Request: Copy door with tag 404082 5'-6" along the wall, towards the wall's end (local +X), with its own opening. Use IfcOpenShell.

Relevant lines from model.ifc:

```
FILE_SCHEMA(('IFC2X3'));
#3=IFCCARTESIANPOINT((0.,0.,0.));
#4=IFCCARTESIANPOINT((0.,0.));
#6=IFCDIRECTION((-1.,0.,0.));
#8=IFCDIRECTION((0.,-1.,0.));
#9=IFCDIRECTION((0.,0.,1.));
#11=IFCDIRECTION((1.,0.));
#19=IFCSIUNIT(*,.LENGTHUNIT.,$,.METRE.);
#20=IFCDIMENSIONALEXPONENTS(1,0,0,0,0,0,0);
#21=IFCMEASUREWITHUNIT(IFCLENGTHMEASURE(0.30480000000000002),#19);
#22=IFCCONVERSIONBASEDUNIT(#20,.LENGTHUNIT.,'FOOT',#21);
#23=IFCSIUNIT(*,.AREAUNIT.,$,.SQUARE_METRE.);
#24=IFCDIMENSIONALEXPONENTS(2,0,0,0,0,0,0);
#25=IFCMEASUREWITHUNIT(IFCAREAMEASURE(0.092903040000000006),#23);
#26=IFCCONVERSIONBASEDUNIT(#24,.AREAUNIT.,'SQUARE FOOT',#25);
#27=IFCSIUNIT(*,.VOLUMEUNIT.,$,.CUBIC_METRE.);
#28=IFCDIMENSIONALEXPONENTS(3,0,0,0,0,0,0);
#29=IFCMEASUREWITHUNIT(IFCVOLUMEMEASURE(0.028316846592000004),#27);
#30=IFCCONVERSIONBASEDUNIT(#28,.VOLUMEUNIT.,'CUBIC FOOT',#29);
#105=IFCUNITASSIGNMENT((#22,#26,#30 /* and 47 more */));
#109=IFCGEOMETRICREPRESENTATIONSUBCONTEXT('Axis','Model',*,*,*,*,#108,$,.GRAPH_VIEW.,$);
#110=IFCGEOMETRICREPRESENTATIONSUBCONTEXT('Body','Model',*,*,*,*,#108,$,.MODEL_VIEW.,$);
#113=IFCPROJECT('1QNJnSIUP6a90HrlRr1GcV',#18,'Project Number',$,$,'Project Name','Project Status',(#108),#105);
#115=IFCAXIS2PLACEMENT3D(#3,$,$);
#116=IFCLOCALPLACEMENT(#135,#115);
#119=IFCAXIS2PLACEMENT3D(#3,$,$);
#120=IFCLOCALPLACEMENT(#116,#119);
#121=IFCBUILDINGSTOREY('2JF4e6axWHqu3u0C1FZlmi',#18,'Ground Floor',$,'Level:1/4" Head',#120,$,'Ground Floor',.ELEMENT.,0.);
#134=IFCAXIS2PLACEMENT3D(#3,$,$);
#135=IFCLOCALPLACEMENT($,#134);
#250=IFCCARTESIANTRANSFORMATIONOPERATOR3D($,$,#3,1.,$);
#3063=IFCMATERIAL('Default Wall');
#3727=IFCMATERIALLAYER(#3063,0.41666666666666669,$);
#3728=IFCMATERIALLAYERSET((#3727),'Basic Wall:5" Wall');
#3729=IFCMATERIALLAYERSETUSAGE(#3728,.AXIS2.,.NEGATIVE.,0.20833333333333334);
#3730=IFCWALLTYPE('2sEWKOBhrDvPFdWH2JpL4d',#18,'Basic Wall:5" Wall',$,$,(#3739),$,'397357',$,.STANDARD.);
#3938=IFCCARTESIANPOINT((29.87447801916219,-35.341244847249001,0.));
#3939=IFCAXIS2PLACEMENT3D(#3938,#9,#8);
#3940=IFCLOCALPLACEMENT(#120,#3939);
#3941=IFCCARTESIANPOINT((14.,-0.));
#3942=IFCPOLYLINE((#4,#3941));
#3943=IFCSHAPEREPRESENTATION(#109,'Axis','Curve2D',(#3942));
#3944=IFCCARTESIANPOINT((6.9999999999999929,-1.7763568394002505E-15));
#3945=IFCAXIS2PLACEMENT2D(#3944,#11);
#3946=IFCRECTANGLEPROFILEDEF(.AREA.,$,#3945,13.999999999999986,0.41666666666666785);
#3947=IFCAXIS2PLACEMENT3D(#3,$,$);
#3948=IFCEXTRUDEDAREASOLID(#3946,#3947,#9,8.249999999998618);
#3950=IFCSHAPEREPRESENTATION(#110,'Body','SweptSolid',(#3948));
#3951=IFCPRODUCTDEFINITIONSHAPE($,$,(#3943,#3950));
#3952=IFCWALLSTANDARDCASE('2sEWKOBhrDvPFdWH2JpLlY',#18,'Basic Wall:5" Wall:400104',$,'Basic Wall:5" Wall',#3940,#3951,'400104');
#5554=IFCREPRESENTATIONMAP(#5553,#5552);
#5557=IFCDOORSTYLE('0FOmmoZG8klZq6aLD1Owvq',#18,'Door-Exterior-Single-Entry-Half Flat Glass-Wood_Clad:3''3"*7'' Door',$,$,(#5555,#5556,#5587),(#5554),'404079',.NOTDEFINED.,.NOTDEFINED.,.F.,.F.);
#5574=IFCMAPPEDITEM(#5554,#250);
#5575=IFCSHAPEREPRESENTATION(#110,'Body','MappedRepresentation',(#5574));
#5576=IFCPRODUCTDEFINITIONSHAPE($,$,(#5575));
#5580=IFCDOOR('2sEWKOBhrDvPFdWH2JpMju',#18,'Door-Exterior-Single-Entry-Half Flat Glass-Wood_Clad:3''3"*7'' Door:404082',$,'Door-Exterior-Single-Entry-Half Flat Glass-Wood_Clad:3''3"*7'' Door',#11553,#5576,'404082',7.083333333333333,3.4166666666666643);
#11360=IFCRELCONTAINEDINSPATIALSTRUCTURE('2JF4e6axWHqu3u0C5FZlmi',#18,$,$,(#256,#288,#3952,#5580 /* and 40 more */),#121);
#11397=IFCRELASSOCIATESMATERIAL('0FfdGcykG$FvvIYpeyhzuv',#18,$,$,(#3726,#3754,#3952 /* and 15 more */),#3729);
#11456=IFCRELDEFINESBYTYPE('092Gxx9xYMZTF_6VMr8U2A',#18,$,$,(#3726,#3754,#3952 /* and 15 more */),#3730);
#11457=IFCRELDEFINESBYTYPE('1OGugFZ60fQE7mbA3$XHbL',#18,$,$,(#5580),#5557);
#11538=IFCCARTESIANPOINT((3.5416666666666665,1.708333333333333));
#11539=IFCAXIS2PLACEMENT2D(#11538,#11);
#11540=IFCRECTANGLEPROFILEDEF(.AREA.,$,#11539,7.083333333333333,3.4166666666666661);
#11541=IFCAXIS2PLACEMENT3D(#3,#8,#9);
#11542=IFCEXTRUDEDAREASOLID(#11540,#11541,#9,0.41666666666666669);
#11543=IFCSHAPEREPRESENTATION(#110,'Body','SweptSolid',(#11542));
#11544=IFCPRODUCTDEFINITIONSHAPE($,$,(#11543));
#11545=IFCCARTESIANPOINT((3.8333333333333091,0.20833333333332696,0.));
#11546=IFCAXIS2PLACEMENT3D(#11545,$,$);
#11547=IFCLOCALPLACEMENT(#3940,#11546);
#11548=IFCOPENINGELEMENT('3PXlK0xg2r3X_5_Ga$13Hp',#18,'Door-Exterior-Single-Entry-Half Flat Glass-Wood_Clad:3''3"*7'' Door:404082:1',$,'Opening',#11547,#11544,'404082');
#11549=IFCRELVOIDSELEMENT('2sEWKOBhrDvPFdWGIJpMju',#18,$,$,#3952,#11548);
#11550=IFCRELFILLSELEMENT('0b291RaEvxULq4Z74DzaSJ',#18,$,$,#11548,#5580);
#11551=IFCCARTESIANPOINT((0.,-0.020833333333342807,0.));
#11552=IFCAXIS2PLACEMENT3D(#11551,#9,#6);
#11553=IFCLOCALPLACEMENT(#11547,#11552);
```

```python
import ifcopenshell
import ifcopenshell.api.feature
import ifcopenshell.api.geometry
import ifcopenshell.api.root
import ifcopenshell.geom
import ifcopenshell.util.element
import ifcopenshell.util.placement
import ifcopenshell.util.shape
import ifcopenshell.util.unit

model = ifcopenshell.open("model.ifc")
unit_scale = ifcopenshell.util.unit.calculate_unit_scale(model)
settings = ifcopenshell.geom.settings()


def volume(element):
    """Net volume in cubic metres, openings subtracted."""
    shape = ifcopenshell.geom.create_shape(settings, element)
    return ifcopenshell.util.shape.get_volume(shape.geometry)


def reuse_history(source, copy):
    """copy_class also copies each property set's owner history, people and application; keep the originals."""
    for rel in copy.IsDefinedBy:
        if rel.is_a("IfcRelDefinesByProperties") and (history := rel.RelatingPropertyDefinition.OwnerHistory):
            rel.RelatingPropertyDefinition.OwnerHistory = source.OwnerHistory
            ifcopenshell.util.element.remove_deep2(model, history)


door = model.by_guid("2sEWKOBhrDvPFdWH2JpMju")
opening = door.FillsVoids[0].RelatingOpeningElement
wall = opening.VoidsElements[0].RelatingBuildingElement
before = volume(wall)
shift = ifcopenshell.util.placement.get_local_placement(wall.ObjectPlacement)[:3, 0] * 66 * 0.0254 / unit_scale

# copy_class copies the void relationship, type, container and properties, but no geometry.
new_opening = ifcopenshell.api.root.copy_class(model, product=opening)
new_opening.Representation = ifcopenshell.util.element.copy_deep(
    model, opening.Representation, exclude=["IfcGeometricRepresentationContext", "IfcRepresentationMap"]
)
new_opening.Name = 'Door-Exterior-Single-Entry-Half Flat Glass-Wood_Clad:3\'3"*7\' Door'
new_opening.Tag = None
new_door = ifcopenshell.api.root.copy_class(model, product=door)
new_door.Representation = ifcopenshell.util.element.copy_deep(
    model, door.Representation, exclude=["IfcGeometricRepresentationContext", "IfcRepresentationMap"]
)
new_door.Name = 'Door-Exterior-Single-Entry-Half Flat Glass-Wood_Clad:3\'3"*7\' Door'
new_door.Tag = None
reuse_history(door, new_door)
fills = ifcopenshell.api.feature.add_filling(model, opening=new_opening, element=new_door)
fills.OwnerHistory = new_door.OwnerHistory  # required in IFC2X3

for old, new in ((opening, new_opening), (door, new_door)):
    matrix = ifcopenshell.util.placement.get_local_placement(old.ObjectPlacement)
    matrix[:3, 3] += shift
    ifcopenshell.api.geometry.edit_object_placement(model, product=new, matrix=matrix, is_si=False)

after = volume(wall)

print(f"wall volume {before:.3f} -> {after:.3f} m3")

model.write("model_updated.ifc")
```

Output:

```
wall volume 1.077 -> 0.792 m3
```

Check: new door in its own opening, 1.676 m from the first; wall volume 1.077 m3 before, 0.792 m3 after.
